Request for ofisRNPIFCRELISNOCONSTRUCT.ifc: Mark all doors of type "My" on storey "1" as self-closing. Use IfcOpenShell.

First a look at what the model holds.

```python
import ifcopenshell
import ifcopenshell.util.element

model = ifcopenshell.open("ofisRNPIFCRELISNOCONSTRUCT.ifc")
print(model.schema)
storey = next(s for s in model.by_type("IfcBuildingStorey") if s.Name == "1")
doors = [e for e in ifcopenshell.util.element.get_decomposition(storey) if e.is_a("IfcDoor")]
seen = {}
for e in doors:
    element_type = ifcopenshell.util.element.get_type(e)
    key = (element_type.Name if element_type != e and element_type else None, ifcopenshell.util.element.get_pset(e, "Pset_DoorCommon", "SelfClosing"))
    seen[key] = seen.get(key, 0) + 1
for (name, value), count in sorted(seen.items(), key=str):
    print(count, "x", name, "|", value)
```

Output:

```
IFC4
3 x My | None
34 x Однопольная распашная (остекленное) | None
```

```python
import ifcopenshell
import ifcopenshell.api.pset
import ifcopenshell.util.element

model = ifcopenshell.open("ofisRNPIFCRELISNOCONSTRUCT.ifc")

storey = next(s for s in model.by_type("IfcBuildingStorey") if s.Name == "1")
doors = [e for e in ifcopenshell.util.element.get_decomposition(storey) if e.is_a("IfcDoor")]

count = 0
for e in doors:
    element_type = ifcopenshell.util.element.get_type(e)
    if element_type in (None, e) or element_type.Name != "My":
        continue
    # add_pset returns the element's existing set when there is one.
    pset = ifcopenshell.api.pset.add_pset(model, product=e, name="Pset_DoorCommon")
    ifcopenshell.api.pset.edit_pset(model, pset=pset, properties={"SelfClosing": True})
    count += 1

print(count, "doors updated")

model.write("ofisRNPIFCRELISNOCONSTRUCT_rev.ifc")
```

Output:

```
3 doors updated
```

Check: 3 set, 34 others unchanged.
